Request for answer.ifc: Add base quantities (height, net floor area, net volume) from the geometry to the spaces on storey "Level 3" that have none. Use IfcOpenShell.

First a look at what the model holds.

```python
import ifcopenshell
import ifcopenshell.util.element
import ifcopenshell.util.unit

model = ifcopenshell.open("answer.ifc")
print(model.schema)
for unit_type in ("LENGTHUNIT", "AREAUNIT", "VOLUMEUNIT"):
    print(unit_type, ifcopenshell.util.unit.calculate_unit_scale(model, unit_type))
storey = next(s for s in model.by_type("IfcBuildingStorey") if s.Name == "Level 3")
spaces = [e for e in ifcopenshell.util.element.get_decomposition(storey) if e.is_a("IfcSpace")]
for e in sorted(spaces, key=lambda e: e.id()):
    print(e.id(), e.is_a(), e.Name, list(ifcopenshell.util.element.get_psets(e, qtos_only=True)), sep=" | ")
```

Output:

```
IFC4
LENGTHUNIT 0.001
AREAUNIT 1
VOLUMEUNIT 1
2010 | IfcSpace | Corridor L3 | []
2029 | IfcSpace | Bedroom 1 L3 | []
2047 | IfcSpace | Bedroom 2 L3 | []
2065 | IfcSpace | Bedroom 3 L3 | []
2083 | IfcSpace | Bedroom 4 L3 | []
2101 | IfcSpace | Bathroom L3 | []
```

```python
import ifcopenshell
import ifcopenshell.api.pset
import ifcopenshell.geom
import ifcopenshell.util.element
import ifcopenshell.util.shape
import ifcopenshell.util.unit

model = ifcopenshell.open("answer.ifc")
unit_scale = ifcopenshell.util.unit.calculate_unit_scale(model)
area_scale = ifcopenshell.util.unit.calculate_unit_scale(model, "AREAUNIT")
volume_scale = ifcopenshell.util.unit.calculate_unit_scale(model, "VOLUMEUNIT")
settings = ifcopenshell.geom.settings()

storey = next(s for s in model.by_type("IfcBuildingStorey") if s.Name == "Level 3")
spaces = [e for e in ifcopenshell.util.element.get_decomposition(storey) if e.is_a("IfcSpace")]

for e in sorted(spaces, key=lambda e: e.id()):
    if ifcopenshell.util.element.get_psets(e, qtos_only=True, should_inherit=False):
        continue
    # Geometry comes back in metres, in the element's own axes.
    shape = ifcopenshell.geom.create_shape(settings, e)
    values = {
        "Height": ifcopenshell.util.shape.get_z(shape.geometry) / unit_scale,
        "NetFloorArea": ifcopenshell.util.shape.get_footprint_area(shape.geometry) / area_scale,
        "NetVolume": ifcopenshell.util.shape.get_volume(shape.geometry) / volume_scale,
    }
    qto = ifcopenshell.api.pset.add_qto(model, product=e, name="Qto_SpaceBaseQuantities")
    ifcopenshell.api.pset.edit_qto(model, qto=qto, properties=values)
    print(e.id(), {k: round(v, 3) for k, v in values.items()})

model.write("answer_updated.ifc")
```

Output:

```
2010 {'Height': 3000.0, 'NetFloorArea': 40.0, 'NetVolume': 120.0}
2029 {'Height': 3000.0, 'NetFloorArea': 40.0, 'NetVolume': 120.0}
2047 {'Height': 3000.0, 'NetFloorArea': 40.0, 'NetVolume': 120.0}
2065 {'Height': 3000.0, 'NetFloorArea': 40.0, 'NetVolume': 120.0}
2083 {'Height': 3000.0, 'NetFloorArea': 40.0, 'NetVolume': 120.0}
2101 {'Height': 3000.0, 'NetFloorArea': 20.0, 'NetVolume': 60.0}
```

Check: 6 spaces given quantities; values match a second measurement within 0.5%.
